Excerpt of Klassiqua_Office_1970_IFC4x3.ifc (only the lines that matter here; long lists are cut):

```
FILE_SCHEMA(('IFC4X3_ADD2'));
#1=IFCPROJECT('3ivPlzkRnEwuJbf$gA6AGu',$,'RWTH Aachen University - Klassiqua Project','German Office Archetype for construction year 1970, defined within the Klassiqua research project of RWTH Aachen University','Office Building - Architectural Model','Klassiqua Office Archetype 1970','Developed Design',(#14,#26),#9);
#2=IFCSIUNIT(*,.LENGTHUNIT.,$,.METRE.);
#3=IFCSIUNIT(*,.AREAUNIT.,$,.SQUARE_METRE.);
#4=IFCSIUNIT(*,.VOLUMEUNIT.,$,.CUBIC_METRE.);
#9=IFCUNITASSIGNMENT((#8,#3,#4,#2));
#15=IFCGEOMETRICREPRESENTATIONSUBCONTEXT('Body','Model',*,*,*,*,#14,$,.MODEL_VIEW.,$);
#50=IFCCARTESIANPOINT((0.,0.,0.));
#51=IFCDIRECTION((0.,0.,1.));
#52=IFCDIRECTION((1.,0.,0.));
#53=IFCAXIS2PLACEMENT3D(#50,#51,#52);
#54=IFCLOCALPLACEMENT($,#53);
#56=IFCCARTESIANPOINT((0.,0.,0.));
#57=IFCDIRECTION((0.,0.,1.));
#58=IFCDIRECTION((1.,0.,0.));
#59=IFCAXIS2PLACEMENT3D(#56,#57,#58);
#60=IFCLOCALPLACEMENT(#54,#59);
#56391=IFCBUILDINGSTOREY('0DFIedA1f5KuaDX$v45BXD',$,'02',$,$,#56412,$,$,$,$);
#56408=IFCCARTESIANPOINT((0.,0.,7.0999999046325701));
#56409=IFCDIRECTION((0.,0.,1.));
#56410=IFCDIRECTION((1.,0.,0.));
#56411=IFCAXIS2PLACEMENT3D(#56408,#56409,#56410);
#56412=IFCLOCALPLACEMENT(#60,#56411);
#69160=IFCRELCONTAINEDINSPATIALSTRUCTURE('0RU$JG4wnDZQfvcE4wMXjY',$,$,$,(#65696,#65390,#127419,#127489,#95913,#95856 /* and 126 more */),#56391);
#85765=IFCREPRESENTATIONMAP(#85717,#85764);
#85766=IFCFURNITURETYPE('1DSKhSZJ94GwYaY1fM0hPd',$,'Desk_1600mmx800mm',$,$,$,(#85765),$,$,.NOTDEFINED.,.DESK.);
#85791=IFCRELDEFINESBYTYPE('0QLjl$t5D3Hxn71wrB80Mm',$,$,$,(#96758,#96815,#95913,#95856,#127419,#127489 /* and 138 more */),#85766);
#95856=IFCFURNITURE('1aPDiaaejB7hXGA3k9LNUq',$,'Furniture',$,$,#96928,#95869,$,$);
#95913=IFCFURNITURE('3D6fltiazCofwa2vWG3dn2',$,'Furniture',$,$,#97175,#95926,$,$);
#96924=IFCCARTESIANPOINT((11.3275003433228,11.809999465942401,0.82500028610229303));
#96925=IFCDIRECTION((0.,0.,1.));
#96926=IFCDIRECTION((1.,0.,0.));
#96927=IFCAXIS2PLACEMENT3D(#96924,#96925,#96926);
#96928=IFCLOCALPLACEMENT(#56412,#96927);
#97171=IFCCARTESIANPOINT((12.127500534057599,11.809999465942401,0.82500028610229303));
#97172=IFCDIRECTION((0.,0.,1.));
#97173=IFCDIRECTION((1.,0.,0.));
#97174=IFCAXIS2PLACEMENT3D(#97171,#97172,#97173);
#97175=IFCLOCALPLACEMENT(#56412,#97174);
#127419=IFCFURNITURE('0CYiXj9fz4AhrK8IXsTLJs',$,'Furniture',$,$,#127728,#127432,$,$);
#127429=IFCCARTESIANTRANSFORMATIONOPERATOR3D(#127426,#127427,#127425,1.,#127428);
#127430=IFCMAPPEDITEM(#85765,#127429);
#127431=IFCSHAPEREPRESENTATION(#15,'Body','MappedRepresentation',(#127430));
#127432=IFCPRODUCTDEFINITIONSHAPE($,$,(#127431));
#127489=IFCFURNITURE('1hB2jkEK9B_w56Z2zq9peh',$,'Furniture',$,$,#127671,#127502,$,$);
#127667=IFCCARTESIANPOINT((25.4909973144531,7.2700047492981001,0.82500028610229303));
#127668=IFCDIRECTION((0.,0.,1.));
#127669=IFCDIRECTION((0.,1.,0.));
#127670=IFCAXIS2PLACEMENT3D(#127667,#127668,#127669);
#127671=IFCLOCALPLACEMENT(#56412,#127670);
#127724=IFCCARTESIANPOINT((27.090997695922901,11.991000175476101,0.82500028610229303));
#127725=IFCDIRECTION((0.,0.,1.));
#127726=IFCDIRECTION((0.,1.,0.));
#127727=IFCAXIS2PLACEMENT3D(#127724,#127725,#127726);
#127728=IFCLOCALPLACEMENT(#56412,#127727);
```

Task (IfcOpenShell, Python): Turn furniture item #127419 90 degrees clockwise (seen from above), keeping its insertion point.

```python
import ifcopenshell
import ifcopenshell.api.geometry
import ifcopenshell.util.placement

model = ifcopenshell.open("Klassiqua_Office_1970_IFC4x3.ifc")

item = model.by_guid("0CYiXj9fz4AhrK8IXsTLJs")
matrix = ifcopenshell.util.placement.get_local_placement(item.ObjectPlacement)
matrix = matrix @ ifcopenshell.util.placement.rotation(-90, "Z")
ifcopenshell.api.geometry.edit_object_placement(model, product=item, matrix=matrix, is_si=False)

print(ifcopenshell.util.placement.get_local_placement(item.ObjectPlacement).round(3) + 0.0)

model.write("Klassiqua_Office_1970_IFC4x3_rev.ifc")
```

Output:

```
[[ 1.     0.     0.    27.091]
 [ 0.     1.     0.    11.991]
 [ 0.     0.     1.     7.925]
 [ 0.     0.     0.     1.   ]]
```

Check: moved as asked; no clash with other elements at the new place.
